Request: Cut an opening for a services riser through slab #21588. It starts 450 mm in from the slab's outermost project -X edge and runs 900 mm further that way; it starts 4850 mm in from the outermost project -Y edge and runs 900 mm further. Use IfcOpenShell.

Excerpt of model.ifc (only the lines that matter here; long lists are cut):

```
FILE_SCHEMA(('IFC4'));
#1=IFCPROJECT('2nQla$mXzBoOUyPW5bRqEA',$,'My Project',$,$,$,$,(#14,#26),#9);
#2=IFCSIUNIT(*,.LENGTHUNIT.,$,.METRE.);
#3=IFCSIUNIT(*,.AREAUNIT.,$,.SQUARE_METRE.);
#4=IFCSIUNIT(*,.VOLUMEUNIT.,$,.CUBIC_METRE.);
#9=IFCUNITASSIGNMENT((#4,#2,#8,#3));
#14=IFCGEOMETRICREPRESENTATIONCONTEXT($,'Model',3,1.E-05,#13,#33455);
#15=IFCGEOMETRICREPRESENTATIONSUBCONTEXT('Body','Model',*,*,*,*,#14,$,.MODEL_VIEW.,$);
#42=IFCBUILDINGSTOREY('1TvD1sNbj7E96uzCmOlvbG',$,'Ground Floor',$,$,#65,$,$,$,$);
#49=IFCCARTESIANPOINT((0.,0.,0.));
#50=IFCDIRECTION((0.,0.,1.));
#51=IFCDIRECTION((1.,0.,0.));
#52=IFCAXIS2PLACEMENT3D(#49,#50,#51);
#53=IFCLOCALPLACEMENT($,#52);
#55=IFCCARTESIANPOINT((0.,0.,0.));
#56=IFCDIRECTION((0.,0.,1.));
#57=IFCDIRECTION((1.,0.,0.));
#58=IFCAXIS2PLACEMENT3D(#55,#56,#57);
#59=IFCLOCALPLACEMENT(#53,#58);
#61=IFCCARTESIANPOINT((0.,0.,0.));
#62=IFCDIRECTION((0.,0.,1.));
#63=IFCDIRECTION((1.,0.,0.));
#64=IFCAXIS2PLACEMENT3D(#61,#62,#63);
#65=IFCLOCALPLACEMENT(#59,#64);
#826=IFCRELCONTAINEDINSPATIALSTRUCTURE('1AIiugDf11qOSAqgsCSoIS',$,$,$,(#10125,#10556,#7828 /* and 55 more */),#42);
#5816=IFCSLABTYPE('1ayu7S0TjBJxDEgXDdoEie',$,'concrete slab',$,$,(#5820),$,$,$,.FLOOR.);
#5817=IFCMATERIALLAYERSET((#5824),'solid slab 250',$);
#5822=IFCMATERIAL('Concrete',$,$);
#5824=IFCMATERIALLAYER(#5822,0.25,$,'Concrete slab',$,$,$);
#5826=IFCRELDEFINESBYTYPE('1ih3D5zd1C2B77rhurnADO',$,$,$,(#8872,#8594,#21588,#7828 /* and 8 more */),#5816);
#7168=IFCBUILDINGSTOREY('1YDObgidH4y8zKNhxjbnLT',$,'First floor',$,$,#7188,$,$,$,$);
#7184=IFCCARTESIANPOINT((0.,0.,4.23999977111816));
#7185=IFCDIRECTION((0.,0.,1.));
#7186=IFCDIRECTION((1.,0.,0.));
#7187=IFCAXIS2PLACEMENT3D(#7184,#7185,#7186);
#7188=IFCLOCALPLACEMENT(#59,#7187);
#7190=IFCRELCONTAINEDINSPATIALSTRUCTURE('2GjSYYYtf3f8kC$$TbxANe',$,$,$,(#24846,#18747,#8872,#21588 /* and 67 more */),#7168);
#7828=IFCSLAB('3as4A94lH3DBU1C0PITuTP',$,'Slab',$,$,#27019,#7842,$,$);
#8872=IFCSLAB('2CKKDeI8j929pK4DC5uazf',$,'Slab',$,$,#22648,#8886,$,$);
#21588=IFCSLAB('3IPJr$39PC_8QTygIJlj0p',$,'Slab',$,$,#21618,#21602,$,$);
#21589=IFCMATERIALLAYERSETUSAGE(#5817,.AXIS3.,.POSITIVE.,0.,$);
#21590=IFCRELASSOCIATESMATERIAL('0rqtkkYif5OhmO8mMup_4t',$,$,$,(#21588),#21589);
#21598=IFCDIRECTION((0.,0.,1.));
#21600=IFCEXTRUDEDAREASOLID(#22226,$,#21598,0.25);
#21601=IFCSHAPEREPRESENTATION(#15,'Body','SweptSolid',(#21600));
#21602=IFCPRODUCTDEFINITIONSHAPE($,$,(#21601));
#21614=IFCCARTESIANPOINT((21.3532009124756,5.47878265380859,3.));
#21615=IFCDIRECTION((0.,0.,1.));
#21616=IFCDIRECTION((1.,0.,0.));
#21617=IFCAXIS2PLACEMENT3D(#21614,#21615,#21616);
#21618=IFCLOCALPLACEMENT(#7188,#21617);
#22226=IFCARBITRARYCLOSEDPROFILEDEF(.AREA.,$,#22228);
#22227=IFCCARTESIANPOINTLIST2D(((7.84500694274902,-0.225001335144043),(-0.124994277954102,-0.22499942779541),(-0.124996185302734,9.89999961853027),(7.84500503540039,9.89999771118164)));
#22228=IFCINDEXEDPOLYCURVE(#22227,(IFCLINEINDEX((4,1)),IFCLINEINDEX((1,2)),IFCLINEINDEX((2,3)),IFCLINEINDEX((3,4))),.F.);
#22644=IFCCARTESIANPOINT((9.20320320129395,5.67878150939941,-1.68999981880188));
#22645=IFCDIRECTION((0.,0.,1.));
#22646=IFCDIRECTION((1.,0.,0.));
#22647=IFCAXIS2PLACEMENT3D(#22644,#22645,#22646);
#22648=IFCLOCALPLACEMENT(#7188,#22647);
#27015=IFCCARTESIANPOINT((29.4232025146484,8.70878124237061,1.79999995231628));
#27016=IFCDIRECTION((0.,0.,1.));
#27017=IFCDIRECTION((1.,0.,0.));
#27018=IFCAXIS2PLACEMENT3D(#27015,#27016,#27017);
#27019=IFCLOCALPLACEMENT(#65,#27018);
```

```python
import numpy as np
import ifcopenshell
import ifcopenshell.api.feature
import ifcopenshell.api.geometry
import ifcopenshell.api.root
import ifcopenshell.geom
import ifcopenshell.util.placement
import ifcopenshell.util.representation
import ifcopenshell.util.shape
import ifcopenshell.util.unit

model = ifcopenshell.open("model.ifc")
unit_scale = ifcopenshell.util.unit.calculate_unit_scale(model)
settings = ifcopenshell.geom.settings()


def volume(element):
    """Net volume in cubic metres, openings subtracted."""
    shape = ifcopenshell.geom.create_shape(settings, element)
    return ifcopenshell.util.shape.get_volume(shape.geometry)


slab = model.by_id(21588)
before = volume(slab)

# Extent in the slab's own axes, in metres. The edges named are its -X and -Y sides.
slab_shape = ifcopenshell.geom.create_shape(settings, slab)
vertices = ifcopenshell.util.shape.get_vertices(slab_shape.geometry)
x_min, y_min, bottom = vertices.min(axis=0)
top = vertices[:, 2].max()

opening = ifcopenshell.api.root.create_entity(model, ifc_class="IfcOpeningElement", name="Services riser opening", predefined_type="OPENING")
context = ifcopenshell.util.representation.get_context(model, "Model", "Body", "MODEL_VIEW")
width, depth = 0.9, 0.9
outline = [(0.0, 0.0), (width, 0.0), (width, depth), (0.0, depth), (0.0, 0.0)]
# Overshoot both faces by 50 mm so the cut is clean.
shape = ifcopenshell.api.geometry.add_slab_representation(
    model, context=context, depth=top - bottom + 0.1, polyline=outline
)
ifcopenshell.api.geometry.assign_representation(model, product=opening, representation=shape)

matrix = ifcopenshell.util.placement.get_local_placement(slab.ObjectPlacement)
matrix[:, 3] = matrix @ np.append(np.array([x_min + 0.45, y_min + 4.85, bottom - 0.05]) / unit_scale, 1.0)
ifcopenshell.api.geometry.edit_object_placement(model, product=opening, matrix=matrix, is_si=False)
ifcopenshell.api.feature.add_feature(model, feature=opening, element=slab)

after = volume(slab)

print(f"slab volume {before:.3f} -> {after:.3f} m3")

model.write("model_rev.ifc")
```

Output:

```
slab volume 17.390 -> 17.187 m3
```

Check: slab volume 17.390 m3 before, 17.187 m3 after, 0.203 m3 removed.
